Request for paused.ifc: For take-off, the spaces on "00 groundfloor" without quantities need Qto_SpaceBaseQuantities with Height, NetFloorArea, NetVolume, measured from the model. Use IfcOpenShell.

First a look at what the model holds.

```python
import ifcopenshell
import ifcopenshell.util.element
import ifcopenshell.util.unit

model = ifcopenshell.open("paused.ifc")
print(model.schema)
for unit_type in ("LENGTHUNIT", "AREAUNIT", "VOLUMEUNIT"):
    print(unit_type, ifcopenshell.util.unit.calculate_unit_scale(model, unit_type))
storey = next(s for s in model.by_type("IfcBuildingStorey") if s.Name == "00 groundfloor")
spaces = [e for e in ifcopenshell.util.element.get_decomposition(storey) if e.is_a("IfcSpace")]
for e in sorted(spaces, key=lambda e: e.id()):
    print(e.id(), e.is_a(), e.Name, list(ifcopenshell.util.element.get_psets(e, qtos_only=True)), sep=" | ")
```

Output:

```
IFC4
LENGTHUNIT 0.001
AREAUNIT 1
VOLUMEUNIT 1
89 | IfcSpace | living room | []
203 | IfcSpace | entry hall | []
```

```python
import ifcopenshell
import ifcopenshell.api.pset
import ifcopenshell.geom
import ifcopenshell.util.element
import ifcopenshell.util.shape
import ifcopenshell.util.unit

model = ifcopenshell.open("paused.ifc")
unit_scale = ifcopenshell.util.unit.calculate_unit_scale(model)
area_scale = ifcopenshell.util.unit.calculate_unit_scale(model, "AREAUNIT")
volume_scale = ifcopenshell.util.unit.calculate_unit_scale(model, "VOLUMEUNIT")
settings = ifcopenshell.geom.settings()

storey = next(s for s in model.by_type("IfcBuildingStorey") if s.Name == "00 groundfloor")
spaces = [e for e in ifcopenshell.util.element.get_decomposition(storey) if e.is_a("IfcSpace")]

for e in sorted(spaces, key=lambda e: e.id()):
    if ifcopenshell.util.element.get_psets(e, qtos_only=True, should_inherit=False):
        continue
    # Geometry comes back in metres, in the element's own axes.
    shape = ifcopenshell.geom.create_shape(settings, e)
    values = {
        "Height": ifcopenshell.util.shape.get_z(shape.geometry) / unit_scale,
        "NetFloorArea": ifcopenshell.util.shape.get_footprint_area(shape.geometry) / area_scale,
        "NetVolume": ifcopenshell.util.shape.get_volume(shape.geometry) / volume_scale,
    }
    qto = ifcopenshell.api.pset.add_qto(model, product=e, name="Qto_SpaceBaseQuantities")
    ifcopenshell.api.pset.edit_qto(model, qto=qto, properties=values)
    print(e.id(), {k: round(v, 3) for k, v in values.items()})

model.write("paused_v2.ifc")
```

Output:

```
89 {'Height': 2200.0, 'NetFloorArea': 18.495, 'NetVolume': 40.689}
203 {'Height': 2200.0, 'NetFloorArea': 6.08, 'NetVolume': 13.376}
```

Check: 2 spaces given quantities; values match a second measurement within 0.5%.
